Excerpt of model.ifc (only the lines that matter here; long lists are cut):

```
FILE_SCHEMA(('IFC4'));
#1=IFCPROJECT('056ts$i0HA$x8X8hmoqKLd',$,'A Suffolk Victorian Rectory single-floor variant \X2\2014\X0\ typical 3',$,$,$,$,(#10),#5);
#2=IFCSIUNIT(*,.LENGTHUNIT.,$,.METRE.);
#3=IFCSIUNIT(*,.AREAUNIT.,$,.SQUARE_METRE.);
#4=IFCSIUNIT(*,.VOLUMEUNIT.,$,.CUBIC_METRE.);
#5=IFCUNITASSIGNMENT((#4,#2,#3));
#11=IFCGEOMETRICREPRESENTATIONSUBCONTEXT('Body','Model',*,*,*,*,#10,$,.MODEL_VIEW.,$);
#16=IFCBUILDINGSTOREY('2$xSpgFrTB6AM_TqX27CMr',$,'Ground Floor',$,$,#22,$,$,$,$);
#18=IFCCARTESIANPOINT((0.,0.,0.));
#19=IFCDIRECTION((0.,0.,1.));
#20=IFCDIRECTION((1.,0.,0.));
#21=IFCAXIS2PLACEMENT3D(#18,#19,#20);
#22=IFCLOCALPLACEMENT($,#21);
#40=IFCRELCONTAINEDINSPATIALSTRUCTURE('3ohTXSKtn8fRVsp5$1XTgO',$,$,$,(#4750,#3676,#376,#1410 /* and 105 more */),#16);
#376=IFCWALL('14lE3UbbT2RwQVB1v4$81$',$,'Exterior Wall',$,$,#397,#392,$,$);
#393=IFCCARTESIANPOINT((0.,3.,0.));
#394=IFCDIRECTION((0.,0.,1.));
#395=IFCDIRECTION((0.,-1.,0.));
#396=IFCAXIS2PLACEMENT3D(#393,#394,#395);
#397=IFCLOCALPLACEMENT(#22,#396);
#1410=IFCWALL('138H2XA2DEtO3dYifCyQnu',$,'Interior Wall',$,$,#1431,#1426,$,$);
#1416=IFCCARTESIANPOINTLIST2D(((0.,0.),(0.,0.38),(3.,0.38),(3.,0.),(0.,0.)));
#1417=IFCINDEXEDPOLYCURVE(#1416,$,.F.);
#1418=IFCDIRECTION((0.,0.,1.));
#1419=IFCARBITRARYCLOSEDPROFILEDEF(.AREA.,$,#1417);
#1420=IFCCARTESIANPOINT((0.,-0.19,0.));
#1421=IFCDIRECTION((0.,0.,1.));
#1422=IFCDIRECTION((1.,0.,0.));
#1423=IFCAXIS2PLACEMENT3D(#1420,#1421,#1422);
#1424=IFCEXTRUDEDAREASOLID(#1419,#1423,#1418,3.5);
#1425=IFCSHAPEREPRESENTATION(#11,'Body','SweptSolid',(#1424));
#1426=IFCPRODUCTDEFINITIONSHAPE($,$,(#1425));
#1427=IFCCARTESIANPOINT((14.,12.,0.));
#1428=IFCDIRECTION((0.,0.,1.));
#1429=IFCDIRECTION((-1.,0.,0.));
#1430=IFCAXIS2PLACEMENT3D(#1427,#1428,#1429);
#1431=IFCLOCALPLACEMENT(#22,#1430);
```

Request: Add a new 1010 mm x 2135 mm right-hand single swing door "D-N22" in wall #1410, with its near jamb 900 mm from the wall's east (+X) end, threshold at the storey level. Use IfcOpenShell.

```python
import numpy as np
import ifcopenshell
import ifcopenshell.api.feature
import ifcopenshell.api.geometry
import ifcopenshell.api.root
import ifcopenshell.api.spatial
import ifcopenshell.geom
import ifcopenshell.util.element
import ifcopenshell.util.placement
import ifcopenshell.util.representation
import ifcopenshell.util.shape
import ifcopenshell.util.unit

model = ifcopenshell.open("model.ifc")
unit_scale = ifcopenshell.util.unit.calculate_unit_scale(model)
settings = ifcopenshell.geom.settings()


def volume(element):
    """Net volume in cubic metres, openings subtracted."""
    shape = ifcopenshell.geom.create_shape(settings, element)
    return ifcopenshell.util.shape.get_volume(shape.geometry)


wall = model.by_id(1410)
storey = ifcopenshell.util.element.get_container(wall, ifc_class="IfcBuildingStorey")
context = ifcopenshell.util.representation.get_context(model, "Model", "Body", "MODEL_VIEW")
before = volume(wall)

width, height, from_end, sill = 1.01, 2.135, 0.9, 0.0  # metres

# The wall runs along its own X axis, and the end named is its -X end.
wall_shape = ifcopenshell.geom.create_shape(settings, wall)
x, y, z = ifcopenshell.util.shape.get_vertices(wall_shape.geometry).T
start = x.min() + from_end
face, thickness = float(y.min()), float(y.max() - y.min())
wall_matrix = ifcopenshell.util.placement.get_local_placement(wall.ObjectPlacement)
level = ifcopenshell.util.placement.get_local_placement(storey.ObjectPlacement)[2, 3]


def in_wall(x, y):
    """Placement at x, y metres in the wall's axes, at sill height."""
    matrix = wall_matrix.copy()
    matrix[:, 3] = wall_matrix @ np.array([x / unit_scale, y / unit_scale, 0.0, 1.0])
    matrix[2, 3] = level + sill / unit_scale
    return matrix


# Opening: a box that overshoots both wall faces by 50 mm.
opening = ifcopenshell.api.root.create_entity(model, ifc_class="IfcOpeningElement", predefined_type="OPENING")
box = ifcopenshell.api.geometry.add_wall_representation(
    model, context=context, length=width, height=height, thickness=thickness + 0.1
)
ifcopenshell.api.geometry.assign_representation(model, product=opening, representation=box)
ifcopenshell.api.geometry.edit_object_placement(model, product=opening, matrix=in_wall(start, face - 0.05), is_si=False)
ifcopenshell.api.feature.add_feature(model, feature=opening, element=wall)

door = ifcopenshell.api.root.create_entity(model, ifc_class="IfcDoor", name="D-N22", predefined_type="DOOR")
door.OverallWidth, door.OverallHeight = width / unit_scale, height / unit_scale
door.OperationType = "SINGLE_SWING_RIGHT"
body = ifcopenshell.api.geometry.add_door_representation(
    model,
    context=context,
    overall_width=door.OverallWidth,
    overall_height=door.OverallHeight,
    operation_type="SINGLE_SWING_RIGHT",
    lining_properties={"LiningDepth": thickness / unit_scale, "ThresholdDepth": thickness / unit_scale},
)
ifcopenshell.api.geometry.assign_representation(model, product=door, representation=body)
ifcopenshell.api.spatial.assign_container(model, products=[door], relating_structure=storey)
ifcopenshell.api.feature.add_filling(model, opening=opening, element=door)

# The lining spans the wall, so the door starts at the wall face.
ifcopenshell.api.geometry.edit_object_placement(model, product=door, matrix=in_wall(start, face), is_si=False)

after = volume(wall)

print(f"wall volume {before:.3f} -> {after:.3f} m3")

model.write("model_v2.ifc")
```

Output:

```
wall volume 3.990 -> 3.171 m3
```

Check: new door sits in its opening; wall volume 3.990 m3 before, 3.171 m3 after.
